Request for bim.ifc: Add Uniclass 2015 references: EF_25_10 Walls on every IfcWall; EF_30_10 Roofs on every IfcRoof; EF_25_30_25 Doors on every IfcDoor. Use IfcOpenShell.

First a look at what the model holds.

```python
import ifcopenshell

model = ifcopenshell.open("bim.ifc")
print(model.schema)
print("classifications:", [c.Name for c in model.by_type("IfcClassification")])
for ifc_class in ("IfcDoor", "IfcRoof", "IfcStair", "IfcWall", "IfcWindow"):
    print(ifc_class, len(model.by_type(ifc_class)))
```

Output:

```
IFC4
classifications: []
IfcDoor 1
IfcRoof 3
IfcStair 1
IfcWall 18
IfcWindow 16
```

```python
import ifcopenshell
import ifcopenshell.api.classification

model = ifcopenshell.open("bim.ifc")

system = ifcopenshell.api.classification.add_classification(model, classification="Uniclass 2015")

codes = {
    "IfcWall": ("EF_25_10", "Walls"),
    "IfcRoof": ("EF_30_10", "Roofs"),
    "IfcDoor": ("EF_25_30_25", "Doors"),
}
for ifc_class, (code, name) in codes.items():
    products = model.by_type(ifc_class)
    ifcopenshell.api.classification.add_reference(
        model, products=products, classification=system, identification=code, name=name
    )
    print(code, len(products))

model.write("bim_rev.ifc")
```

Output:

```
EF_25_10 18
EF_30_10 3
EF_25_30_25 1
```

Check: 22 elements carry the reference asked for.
